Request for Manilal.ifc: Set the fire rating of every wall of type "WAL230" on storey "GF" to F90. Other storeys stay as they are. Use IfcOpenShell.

First a look at what the model holds.

```python
import ifcopenshell
import ifcopenshell.util.element

model = ifcopenshell.open("Manilal.ifc")
print(model.schema)
storey = next(s for s in model.by_type("IfcBuildingStorey") if s.Name == "GF")
walls = [e for e in ifcopenshell.util.element.get_decomposition(storey) if e.is_a("IfcWall")]
seen = {}
for e in walls:
    element_type = ifcopenshell.util.element.get_type(e)
    key = (element_type.Name if element_type != e and element_type else None, ifcopenshell.util.element.get_pset(e, "Pset_WallCommon", "FireRating"))
    seen[key] = seen.get(key, 0) + 1
for (name, value), count in sorted(seen.items(), key=str):
    print(count, "x", name, "|", value)
```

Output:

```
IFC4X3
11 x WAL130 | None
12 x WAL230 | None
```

```python
import ifcopenshell
import ifcopenshell.api.pset
import ifcopenshell.util.element

model = ifcopenshell.open("Manilal.ifc")

storey = next(s for s in model.by_type("IfcBuildingStorey") if s.Name == "GF")
walls = [e for e in ifcopenshell.util.element.get_decomposition(storey) if e.is_a("IfcWall")]

count = 0
for e in walls:
    element_type = ifcopenshell.util.element.get_type(e)
    if element_type in (None, e) or element_type.Name != "WAL230":
        continue
    # add_pset returns the element's existing set when there is one.
    pset = ifcopenshell.api.pset.add_pset(model, product=e, name="Pset_WallCommon")
    ifcopenshell.api.pset.edit_pset(model, pset=pset, properties={"FireRating": "F90"})
    count += 1

print(count, "walls updated")

model.write("Manilal_v2.ifc")
```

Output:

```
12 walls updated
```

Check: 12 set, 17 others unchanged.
